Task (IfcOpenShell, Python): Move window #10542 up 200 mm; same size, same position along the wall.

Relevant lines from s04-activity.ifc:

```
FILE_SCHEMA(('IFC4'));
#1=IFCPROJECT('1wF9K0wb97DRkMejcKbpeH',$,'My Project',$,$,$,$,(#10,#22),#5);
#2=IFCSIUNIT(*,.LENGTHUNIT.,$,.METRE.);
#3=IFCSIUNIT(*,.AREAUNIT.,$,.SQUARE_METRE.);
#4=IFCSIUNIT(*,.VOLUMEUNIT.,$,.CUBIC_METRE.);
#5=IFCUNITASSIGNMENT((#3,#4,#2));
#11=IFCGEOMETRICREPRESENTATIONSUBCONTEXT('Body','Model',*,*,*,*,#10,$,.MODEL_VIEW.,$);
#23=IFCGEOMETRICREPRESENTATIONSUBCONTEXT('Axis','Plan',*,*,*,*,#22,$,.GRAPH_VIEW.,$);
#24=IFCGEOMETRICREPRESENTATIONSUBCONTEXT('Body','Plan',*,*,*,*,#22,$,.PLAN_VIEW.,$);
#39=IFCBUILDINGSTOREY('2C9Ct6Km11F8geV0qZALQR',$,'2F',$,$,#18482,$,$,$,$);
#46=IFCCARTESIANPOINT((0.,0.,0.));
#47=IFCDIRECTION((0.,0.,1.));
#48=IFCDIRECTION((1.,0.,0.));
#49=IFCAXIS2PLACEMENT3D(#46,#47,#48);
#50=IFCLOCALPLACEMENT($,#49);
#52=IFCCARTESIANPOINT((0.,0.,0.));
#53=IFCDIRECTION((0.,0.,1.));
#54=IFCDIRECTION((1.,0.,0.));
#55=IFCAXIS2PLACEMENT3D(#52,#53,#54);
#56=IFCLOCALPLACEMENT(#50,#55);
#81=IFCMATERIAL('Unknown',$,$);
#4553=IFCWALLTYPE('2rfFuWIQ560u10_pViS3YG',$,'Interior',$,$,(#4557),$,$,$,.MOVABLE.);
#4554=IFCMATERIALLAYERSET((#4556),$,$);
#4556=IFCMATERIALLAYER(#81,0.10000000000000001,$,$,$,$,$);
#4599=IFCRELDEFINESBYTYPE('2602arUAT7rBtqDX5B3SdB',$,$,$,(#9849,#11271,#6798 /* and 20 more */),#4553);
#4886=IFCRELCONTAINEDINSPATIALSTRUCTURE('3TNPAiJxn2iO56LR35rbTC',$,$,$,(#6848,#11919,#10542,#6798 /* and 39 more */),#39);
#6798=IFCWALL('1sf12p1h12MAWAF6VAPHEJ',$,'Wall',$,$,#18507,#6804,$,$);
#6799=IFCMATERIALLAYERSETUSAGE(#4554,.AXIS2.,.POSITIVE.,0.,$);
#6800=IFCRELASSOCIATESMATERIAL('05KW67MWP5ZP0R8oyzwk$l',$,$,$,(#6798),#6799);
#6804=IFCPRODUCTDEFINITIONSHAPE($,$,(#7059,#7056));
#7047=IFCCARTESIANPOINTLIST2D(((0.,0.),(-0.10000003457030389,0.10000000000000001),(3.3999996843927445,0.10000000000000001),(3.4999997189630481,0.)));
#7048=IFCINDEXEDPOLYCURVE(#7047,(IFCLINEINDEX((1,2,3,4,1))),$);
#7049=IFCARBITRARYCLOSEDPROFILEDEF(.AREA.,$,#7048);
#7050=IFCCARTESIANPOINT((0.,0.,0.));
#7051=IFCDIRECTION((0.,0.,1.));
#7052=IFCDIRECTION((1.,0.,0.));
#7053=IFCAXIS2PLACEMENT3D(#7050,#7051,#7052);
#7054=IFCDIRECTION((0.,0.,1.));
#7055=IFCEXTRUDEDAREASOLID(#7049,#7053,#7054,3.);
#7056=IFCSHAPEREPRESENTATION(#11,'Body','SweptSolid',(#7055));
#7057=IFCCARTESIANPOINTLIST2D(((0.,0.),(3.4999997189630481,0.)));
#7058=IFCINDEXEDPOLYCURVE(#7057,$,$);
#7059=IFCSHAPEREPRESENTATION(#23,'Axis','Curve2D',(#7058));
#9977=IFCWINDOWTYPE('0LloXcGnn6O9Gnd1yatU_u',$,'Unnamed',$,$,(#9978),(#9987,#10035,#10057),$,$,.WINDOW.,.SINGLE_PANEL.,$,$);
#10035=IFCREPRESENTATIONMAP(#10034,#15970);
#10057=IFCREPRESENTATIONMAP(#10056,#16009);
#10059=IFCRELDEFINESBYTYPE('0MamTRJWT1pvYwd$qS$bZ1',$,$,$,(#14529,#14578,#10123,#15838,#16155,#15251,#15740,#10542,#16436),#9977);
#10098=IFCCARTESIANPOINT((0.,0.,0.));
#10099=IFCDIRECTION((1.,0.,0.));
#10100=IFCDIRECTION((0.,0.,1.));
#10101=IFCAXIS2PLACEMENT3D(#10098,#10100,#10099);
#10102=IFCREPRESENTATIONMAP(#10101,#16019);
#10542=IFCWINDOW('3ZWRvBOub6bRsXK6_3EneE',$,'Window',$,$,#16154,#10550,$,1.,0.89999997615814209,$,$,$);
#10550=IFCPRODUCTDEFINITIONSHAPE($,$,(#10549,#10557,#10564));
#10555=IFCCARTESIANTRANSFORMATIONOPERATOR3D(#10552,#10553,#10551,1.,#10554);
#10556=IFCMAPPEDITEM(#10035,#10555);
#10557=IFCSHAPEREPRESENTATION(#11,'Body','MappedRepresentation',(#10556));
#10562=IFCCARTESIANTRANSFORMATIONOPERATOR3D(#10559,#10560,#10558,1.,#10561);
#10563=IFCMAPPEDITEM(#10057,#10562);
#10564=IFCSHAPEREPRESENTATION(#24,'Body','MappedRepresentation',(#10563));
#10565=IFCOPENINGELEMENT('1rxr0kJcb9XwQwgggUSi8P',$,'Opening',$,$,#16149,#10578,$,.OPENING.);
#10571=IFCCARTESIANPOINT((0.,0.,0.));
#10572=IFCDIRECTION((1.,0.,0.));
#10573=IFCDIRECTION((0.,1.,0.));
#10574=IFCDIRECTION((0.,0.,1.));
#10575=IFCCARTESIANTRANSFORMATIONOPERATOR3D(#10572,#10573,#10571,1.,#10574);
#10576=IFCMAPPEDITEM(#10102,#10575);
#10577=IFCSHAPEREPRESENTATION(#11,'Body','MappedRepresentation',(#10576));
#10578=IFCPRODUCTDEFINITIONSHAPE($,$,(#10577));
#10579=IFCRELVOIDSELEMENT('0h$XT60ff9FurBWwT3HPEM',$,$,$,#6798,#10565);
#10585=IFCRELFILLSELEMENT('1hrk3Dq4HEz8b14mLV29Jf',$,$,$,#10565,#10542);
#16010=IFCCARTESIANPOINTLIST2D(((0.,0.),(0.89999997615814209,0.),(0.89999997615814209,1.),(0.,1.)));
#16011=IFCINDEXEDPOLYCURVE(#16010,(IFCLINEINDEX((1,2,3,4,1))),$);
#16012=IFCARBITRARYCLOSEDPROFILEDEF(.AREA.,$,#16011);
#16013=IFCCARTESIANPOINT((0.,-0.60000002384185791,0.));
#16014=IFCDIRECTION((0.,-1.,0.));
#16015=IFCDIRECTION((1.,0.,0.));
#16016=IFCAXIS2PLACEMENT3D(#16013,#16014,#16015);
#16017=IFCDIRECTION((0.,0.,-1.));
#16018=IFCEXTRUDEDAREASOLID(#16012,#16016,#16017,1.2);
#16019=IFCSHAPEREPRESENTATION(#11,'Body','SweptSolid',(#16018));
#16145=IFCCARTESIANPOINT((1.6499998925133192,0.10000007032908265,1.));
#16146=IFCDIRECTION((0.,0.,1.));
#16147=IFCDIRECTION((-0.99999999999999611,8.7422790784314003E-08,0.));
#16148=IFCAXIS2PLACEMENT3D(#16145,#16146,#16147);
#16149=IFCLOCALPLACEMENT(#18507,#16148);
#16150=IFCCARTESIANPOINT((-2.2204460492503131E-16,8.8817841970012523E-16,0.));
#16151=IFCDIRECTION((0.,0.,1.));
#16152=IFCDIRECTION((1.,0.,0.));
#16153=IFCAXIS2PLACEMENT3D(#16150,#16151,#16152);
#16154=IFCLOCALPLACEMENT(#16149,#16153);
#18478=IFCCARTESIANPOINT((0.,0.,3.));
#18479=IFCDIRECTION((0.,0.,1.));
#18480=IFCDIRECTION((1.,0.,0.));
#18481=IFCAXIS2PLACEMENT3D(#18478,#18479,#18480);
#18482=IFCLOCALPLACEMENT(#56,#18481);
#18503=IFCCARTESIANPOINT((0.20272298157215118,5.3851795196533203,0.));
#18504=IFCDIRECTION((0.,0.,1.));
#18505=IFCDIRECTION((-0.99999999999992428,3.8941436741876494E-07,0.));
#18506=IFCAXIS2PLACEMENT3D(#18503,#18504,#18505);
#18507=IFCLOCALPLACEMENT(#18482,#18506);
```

```python
import numpy as np
import ifcopenshell
import ifcopenshell.api.geometry
import ifcopenshell.util.placement
import ifcopenshell.util.unit

model = ifcopenshell.open("s04-activity.ifc")
unit_scale = ifcopenshell.util.unit.calculate_unit_scale(model)

window = model.by_guid("3ZWRvBOub6bRsXK6_3EneE")
opening = window.FillsVoids[0].RelatingOpeningElement
dz = 0.2 / unit_scale

shift = np.array([0.0, 0.0, dz])
# The window is placed relative to its opening, so it follows when the opening moves.
matrix = ifcopenshell.util.placement.get_local_placement(opening.ObjectPlacement)
matrix[:3, 3] += shift
ifcopenshell.api.geometry.edit_object_placement(
    model, product=opening, matrix=matrix, is_si=False, should_transform_children=True
)

print(f"moved by {dz * unit_scale:+.3f} m")

model.write("s04-activity_rev.ifc")
```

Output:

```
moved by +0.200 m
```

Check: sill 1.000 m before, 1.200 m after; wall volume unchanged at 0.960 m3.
